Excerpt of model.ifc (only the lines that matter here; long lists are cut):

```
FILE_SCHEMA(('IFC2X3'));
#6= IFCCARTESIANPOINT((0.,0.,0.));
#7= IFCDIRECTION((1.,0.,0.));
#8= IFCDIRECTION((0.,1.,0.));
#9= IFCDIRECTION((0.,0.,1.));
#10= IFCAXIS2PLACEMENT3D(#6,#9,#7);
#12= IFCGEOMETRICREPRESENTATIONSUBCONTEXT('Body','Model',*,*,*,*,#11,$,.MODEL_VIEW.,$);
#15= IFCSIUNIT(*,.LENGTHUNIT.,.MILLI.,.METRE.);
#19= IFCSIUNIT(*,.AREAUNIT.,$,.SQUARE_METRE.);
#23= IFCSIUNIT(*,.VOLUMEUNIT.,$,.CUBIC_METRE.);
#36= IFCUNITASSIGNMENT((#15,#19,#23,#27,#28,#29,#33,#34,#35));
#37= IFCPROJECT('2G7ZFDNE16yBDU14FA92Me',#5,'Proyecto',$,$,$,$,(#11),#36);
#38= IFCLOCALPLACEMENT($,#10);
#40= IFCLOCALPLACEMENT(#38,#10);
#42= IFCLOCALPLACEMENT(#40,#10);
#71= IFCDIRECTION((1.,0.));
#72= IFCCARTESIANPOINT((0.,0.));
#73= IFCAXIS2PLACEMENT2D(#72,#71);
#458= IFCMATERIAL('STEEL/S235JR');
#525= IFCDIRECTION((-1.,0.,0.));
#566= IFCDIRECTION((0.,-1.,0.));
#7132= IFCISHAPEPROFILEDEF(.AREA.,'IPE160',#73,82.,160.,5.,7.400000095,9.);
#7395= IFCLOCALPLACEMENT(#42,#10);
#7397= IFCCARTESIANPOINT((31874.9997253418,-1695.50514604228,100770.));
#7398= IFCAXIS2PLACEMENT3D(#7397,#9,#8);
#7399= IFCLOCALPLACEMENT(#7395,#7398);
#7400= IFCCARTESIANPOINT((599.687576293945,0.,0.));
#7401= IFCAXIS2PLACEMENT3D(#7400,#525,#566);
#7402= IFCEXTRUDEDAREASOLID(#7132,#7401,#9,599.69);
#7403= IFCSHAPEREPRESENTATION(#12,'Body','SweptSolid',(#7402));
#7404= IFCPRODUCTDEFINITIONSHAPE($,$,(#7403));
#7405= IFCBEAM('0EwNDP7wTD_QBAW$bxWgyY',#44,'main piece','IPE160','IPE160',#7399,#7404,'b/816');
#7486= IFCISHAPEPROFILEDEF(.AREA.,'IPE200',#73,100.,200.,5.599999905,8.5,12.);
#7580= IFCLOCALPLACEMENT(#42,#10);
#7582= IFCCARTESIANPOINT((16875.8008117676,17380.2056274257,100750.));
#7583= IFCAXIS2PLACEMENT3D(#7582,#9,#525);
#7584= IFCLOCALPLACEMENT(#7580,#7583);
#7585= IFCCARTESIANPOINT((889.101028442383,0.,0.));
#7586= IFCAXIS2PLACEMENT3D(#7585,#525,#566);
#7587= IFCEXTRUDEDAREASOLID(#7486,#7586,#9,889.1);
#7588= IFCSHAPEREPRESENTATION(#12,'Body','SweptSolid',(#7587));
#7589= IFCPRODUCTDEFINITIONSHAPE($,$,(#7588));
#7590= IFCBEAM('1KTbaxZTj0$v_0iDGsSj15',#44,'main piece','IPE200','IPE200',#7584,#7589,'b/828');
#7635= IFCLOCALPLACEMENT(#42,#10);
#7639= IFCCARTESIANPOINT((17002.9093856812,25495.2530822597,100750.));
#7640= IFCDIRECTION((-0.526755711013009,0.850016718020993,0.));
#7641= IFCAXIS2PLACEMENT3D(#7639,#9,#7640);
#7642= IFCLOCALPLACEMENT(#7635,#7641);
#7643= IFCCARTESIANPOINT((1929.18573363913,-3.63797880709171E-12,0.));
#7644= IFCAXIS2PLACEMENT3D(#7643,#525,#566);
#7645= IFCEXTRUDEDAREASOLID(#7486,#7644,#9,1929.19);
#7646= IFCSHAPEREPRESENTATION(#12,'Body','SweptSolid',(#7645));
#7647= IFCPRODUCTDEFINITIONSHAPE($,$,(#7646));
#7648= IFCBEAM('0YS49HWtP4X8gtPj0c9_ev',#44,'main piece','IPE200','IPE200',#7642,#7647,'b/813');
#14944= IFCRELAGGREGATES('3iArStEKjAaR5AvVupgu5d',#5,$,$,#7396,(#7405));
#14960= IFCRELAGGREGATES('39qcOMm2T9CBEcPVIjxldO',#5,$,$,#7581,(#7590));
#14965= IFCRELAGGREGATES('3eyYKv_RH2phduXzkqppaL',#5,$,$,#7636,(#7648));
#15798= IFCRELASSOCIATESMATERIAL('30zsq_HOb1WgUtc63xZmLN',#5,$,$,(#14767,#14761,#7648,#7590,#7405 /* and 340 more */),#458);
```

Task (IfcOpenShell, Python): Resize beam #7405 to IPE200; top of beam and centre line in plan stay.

```python
import ifcopenshell
import ifcopenshell.util.element
import ifcopenshell.util.representation

model = ifcopenshell.open("model.ifc")

member = model.by_guid("0EwNDP7wTD_QBAW$bxWgyY")
source = next(p for p in model.by_type("IfcIShapeProfileDef") if p.ProfileName == "IPE200")

body = ifcopenshell.util.representation.get_representation(member, "Model", "Body")
solid = body.Items[0]
old_profile = solid.SweptArea

# Copy the section's sizes but keep this member's own profile position.
profile = ifcopenshell.util.element.copy(model, source)
# Profiles are centred, so shift by half the change in depth to hold the top.
shift = (old_profile.OverallDepth - profile.OverallDepth) / 2
x, y = old_profile.Position.Location.Coordinates
up = (0.0, 1.0)  # upwards, in the solid's own plane
location = model.createIfcCartesianPoint((x + up[0] * shift, y + up[1] * shift))
profile.Position = model.createIfcAxis2Placement2D(location, old_profile.Position.RefDirection)
solid.SweptArea = profile
if not model.get_total_inverses(old_profile):
    ifcopenshell.util.element.remove_deep2(model, old_profile)
member.Description = member.Description.replace("IPE160", "IPE200")
member.ObjectType = member.ObjectType.replace("IPE160", "IPE200")

print(solid.SweptArea)

model.write("model_v2.ifc")
```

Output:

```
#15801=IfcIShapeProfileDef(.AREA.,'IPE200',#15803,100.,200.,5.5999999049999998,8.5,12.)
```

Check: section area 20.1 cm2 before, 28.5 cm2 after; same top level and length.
